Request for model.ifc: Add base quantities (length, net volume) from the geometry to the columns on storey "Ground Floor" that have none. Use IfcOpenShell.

First a look at what the model holds.

```python
import ifcopenshell
import ifcopenshell.util.element
import ifcopenshell.util.unit

model = ifcopenshell.open("model.ifc")
print(model.schema)
for unit_type in ("LENGTHUNIT", "AREAUNIT", "VOLUMEUNIT"):
    print(unit_type, ifcopenshell.util.unit.calculate_unit_scale(model, unit_type))
storey = next(s for s in model.by_type("IfcBuildingStorey") if s.Name == "Ground Floor")
columns = [e for e in ifcopenshell.util.element.get_decomposition(storey) if e.is_a("IfcColumn")]
for e in sorted(columns, key=lambda e: e.id()):
    print(e.id(), e.is_a(), e.Name, list(ifcopenshell.util.element.get_psets(e, qtos_only=True)), sep=" | ")
```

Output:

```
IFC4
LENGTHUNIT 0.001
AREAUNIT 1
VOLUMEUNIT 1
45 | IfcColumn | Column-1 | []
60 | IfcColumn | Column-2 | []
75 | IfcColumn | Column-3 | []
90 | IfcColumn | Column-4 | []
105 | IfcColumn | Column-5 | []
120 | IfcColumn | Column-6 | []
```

```python
import ifcopenshell
import ifcopenshell.api.pset
import ifcopenshell.geom
import ifcopenshell.util.element
import ifcopenshell.util.shape
import ifcopenshell.util.unit

model = ifcopenshell.open("model.ifc")
unit_scale = ifcopenshell.util.unit.calculate_unit_scale(model)
volume_scale = ifcopenshell.util.unit.calculate_unit_scale(model, "VOLUMEUNIT")
settings = ifcopenshell.geom.settings()

storey = next(s for s in model.by_type("IfcBuildingStorey") if s.Name == "Ground Floor")
columns = [e for e in ifcopenshell.util.element.get_decomposition(storey) if e.is_a("IfcColumn")]

for e in sorted(columns, key=lambda e: e.id()):
    if ifcopenshell.util.element.get_psets(e, qtos_only=True, should_inherit=False):
        continue
    # Geometry comes back in metres, in the element's own axes.
    shape = ifcopenshell.geom.create_shape(settings, e)
    values = {
        "Length": ifcopenshell.util.shape.get_z(shape.geometry) / unit_scale,
        "NetVolume": ifcopenshell.util.shape.get_volume(shape.geometry) / volume_scale,
    }
    qto = ifcopenshell.api.pset.add_qto(model, product=e, name="Qto_ColumnBaseQuantities")
    ifcopenshell.api.pset.edit_qto(model, qto=qto, properties=values)
    print(e.id(), {k: round(v, 3) for k, v in values.items()})

model.write("model_updated.ifc")
```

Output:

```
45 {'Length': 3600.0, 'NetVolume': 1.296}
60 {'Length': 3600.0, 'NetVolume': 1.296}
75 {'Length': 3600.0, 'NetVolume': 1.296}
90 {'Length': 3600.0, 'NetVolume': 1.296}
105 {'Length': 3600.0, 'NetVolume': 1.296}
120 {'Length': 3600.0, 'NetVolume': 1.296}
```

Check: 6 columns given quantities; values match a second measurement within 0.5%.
